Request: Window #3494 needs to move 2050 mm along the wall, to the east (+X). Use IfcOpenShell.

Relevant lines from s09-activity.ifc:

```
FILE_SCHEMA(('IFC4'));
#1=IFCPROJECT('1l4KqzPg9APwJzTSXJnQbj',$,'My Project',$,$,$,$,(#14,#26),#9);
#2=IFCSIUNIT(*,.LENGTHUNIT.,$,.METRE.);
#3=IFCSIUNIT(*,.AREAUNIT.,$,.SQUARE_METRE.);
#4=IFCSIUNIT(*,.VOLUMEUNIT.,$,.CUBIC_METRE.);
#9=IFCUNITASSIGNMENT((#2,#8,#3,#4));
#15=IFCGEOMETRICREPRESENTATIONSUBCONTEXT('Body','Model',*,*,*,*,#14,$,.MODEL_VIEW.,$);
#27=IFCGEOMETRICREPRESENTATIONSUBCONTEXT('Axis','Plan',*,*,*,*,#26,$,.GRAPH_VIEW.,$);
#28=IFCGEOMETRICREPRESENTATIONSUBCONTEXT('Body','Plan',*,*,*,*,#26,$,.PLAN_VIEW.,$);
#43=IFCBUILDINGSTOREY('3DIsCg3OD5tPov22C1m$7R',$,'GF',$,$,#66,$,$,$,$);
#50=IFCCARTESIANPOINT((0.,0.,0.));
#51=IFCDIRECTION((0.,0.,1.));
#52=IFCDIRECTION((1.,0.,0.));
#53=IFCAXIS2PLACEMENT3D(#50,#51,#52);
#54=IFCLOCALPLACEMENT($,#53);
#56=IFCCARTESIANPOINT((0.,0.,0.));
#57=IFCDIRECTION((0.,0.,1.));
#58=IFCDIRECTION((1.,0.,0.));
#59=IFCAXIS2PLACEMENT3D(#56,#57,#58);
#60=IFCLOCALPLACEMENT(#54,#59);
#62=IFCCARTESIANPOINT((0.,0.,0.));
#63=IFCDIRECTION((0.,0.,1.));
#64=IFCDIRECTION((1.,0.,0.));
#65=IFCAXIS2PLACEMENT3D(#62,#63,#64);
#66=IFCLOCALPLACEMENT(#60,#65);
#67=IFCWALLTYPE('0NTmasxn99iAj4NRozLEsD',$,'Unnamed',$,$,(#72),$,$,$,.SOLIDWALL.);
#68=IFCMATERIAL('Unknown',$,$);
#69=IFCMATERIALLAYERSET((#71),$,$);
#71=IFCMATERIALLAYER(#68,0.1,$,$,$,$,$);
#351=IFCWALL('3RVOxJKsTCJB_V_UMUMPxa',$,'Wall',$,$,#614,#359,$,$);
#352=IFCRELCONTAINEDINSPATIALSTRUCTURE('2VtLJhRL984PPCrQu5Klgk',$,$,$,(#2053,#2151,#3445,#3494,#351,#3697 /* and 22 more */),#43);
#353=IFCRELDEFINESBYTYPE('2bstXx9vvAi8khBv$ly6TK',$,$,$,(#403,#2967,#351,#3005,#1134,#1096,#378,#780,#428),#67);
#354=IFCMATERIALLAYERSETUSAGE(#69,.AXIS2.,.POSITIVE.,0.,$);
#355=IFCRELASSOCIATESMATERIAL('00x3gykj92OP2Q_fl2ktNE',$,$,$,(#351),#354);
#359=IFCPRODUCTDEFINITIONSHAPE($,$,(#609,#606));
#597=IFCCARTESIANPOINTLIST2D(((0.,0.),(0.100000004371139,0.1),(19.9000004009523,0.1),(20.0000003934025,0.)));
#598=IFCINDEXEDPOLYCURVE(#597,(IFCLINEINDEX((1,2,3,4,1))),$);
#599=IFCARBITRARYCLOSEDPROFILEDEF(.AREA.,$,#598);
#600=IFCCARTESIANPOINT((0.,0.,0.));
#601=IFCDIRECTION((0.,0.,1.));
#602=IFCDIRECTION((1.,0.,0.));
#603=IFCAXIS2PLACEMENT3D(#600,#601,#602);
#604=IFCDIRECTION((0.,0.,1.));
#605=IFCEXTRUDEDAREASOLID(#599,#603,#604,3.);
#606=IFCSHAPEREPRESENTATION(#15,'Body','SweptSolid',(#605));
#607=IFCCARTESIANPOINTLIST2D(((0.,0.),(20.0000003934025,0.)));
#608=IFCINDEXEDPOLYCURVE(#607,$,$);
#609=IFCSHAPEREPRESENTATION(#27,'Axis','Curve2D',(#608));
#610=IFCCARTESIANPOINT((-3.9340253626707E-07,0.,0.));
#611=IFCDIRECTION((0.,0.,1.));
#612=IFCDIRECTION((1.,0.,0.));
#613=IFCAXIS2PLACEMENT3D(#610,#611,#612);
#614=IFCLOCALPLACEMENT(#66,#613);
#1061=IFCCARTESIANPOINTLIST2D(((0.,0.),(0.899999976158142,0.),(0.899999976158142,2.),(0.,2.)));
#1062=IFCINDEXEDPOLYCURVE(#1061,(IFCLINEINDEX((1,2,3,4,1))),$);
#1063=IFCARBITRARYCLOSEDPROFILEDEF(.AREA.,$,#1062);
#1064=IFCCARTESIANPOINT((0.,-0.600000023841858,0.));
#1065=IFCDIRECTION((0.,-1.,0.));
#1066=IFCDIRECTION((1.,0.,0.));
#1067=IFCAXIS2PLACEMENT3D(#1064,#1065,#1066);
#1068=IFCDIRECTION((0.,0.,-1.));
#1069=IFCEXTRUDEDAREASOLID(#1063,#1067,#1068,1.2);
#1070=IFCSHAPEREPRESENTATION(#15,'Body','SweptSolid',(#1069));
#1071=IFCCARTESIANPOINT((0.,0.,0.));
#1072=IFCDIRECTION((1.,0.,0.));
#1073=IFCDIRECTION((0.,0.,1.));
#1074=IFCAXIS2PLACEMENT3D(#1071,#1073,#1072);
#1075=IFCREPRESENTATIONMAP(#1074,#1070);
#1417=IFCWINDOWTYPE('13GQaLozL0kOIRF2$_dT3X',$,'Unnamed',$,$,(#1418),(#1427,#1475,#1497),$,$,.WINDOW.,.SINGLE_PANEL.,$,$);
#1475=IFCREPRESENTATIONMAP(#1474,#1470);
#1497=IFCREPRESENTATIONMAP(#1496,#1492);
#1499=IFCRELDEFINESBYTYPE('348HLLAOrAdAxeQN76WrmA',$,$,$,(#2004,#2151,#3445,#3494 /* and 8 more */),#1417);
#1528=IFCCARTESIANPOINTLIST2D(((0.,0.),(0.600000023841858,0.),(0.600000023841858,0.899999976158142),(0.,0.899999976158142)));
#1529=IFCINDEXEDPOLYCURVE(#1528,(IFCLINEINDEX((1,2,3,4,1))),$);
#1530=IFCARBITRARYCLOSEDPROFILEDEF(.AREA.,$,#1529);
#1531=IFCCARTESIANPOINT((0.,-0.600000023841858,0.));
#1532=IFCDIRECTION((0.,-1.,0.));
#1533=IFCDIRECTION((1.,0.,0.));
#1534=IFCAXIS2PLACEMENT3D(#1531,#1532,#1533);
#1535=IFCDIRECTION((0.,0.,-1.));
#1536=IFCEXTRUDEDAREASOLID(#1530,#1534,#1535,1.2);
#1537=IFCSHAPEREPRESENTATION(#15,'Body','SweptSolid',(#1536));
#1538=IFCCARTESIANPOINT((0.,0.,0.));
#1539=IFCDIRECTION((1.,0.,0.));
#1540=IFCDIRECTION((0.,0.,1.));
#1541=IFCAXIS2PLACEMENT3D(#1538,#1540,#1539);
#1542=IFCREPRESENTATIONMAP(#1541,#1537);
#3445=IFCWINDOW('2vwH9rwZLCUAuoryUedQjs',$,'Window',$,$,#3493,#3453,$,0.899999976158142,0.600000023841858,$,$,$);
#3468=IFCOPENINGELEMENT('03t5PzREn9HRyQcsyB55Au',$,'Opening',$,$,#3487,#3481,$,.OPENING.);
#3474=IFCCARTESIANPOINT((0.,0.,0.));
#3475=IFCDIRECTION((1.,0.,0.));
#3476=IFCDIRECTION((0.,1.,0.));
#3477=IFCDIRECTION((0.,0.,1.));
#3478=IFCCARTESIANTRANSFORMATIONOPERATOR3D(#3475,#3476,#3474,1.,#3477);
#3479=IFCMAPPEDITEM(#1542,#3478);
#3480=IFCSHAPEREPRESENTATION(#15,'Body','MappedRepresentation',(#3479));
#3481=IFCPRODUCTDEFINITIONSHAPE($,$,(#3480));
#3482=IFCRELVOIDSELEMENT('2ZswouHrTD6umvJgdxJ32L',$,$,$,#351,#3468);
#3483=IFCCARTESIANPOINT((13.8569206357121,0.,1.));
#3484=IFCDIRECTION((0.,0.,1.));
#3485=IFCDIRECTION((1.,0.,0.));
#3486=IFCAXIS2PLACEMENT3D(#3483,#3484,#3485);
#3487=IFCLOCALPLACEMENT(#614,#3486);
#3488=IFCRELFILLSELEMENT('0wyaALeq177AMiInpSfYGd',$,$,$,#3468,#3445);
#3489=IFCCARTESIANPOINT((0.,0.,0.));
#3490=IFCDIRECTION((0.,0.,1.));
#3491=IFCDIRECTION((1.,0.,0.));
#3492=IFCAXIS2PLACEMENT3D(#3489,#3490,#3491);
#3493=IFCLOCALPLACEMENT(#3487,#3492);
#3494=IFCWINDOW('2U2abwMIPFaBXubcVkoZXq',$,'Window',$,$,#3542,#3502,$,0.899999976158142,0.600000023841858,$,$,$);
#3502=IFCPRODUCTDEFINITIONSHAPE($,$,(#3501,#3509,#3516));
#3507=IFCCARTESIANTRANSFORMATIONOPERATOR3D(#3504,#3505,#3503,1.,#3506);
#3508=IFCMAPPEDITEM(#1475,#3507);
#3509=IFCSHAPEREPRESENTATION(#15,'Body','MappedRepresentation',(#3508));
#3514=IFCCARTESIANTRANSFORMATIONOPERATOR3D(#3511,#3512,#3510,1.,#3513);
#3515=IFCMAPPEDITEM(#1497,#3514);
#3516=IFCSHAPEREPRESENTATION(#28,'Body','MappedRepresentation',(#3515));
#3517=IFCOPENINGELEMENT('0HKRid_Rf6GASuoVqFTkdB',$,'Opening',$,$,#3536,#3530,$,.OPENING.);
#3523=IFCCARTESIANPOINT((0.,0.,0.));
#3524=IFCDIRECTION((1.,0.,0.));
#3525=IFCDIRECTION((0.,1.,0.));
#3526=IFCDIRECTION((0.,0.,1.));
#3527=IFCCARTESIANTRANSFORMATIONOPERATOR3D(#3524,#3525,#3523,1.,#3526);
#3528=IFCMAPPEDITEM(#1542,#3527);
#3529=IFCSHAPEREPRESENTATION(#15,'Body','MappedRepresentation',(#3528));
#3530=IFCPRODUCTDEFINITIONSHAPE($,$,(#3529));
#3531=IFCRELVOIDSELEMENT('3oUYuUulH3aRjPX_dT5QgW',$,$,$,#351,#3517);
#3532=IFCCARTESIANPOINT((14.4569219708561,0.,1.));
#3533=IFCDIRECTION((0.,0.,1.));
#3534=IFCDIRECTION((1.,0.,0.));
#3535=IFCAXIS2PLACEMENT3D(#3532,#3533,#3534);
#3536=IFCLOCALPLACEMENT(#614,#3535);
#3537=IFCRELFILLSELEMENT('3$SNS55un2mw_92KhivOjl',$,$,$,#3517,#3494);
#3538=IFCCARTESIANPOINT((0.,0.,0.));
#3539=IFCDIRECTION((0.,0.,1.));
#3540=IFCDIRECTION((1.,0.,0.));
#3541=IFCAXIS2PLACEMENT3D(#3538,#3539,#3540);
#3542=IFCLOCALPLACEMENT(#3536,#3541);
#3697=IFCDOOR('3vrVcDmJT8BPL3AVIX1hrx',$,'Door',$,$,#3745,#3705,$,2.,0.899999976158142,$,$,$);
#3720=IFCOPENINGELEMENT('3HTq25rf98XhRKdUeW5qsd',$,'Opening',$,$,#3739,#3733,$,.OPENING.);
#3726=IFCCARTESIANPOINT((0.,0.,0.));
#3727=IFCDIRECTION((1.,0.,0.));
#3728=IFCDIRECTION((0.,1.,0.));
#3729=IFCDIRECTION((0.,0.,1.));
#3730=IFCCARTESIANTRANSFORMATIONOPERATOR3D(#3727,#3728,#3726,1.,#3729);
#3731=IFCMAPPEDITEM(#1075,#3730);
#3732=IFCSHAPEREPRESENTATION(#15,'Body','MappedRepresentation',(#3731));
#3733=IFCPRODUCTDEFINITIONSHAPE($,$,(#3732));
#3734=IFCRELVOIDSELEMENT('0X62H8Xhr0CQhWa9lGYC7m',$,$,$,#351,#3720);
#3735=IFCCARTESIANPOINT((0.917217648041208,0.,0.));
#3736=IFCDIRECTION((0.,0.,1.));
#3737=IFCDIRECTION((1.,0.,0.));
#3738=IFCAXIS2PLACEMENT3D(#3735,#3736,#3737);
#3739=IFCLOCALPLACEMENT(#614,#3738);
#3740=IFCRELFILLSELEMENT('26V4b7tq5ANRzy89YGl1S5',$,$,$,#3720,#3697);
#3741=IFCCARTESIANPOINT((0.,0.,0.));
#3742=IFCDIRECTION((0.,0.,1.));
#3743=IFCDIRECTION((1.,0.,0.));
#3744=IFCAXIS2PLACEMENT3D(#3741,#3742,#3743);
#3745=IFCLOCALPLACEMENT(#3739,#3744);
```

```python
import ifcopenshell
import ifcopenshell.api.geometry
import ifcopenshell.util.placement
import ifcopenshell.util.unit

model = ifcopenshell.open("s09-activity.ifc")
unit_scale = ifcopenshell.util.unit.calculate_unit_scale(model)

window = model.by_guid("2U2abwMIPFaBXubcVkoZXq")
opening = window.FillsVoids[0].RelatingOpeningElement
wall = opening.VoidsElements[0].RelatingBuildingElement

wall_matrix = ifcopenshell.util.placement.get_local_placement(wall.ObjectPlacement)
shift = wall_matrix[:3, 0] * 2.05 / unit_scale
before = ifcopenshell.util.placement.get_local_placement(window.ObjectPlacement)[:3, 3].copy()

# The window is placed relative to its opening, so it follows when the opening moves.
matrix = ifcopenshell.util.placement.get_local_placement(opening.ObjectPlacement)
matrix[:3, 3] += shift
ifcopenshell.api.geometry.edit_object_placement(
    model, product=opening, matrix=matrix, is_si=False, should_transform_children=True
)

after = ifcopenshell.util.placement.get_local_placement(window.ObjectPlacement)[:3, 3]
print("window moved by", (after - before).round(3) + 0.0)

model.write("s09-activity_rev.ifc")
```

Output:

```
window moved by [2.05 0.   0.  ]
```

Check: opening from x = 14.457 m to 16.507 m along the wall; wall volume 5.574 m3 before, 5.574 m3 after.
